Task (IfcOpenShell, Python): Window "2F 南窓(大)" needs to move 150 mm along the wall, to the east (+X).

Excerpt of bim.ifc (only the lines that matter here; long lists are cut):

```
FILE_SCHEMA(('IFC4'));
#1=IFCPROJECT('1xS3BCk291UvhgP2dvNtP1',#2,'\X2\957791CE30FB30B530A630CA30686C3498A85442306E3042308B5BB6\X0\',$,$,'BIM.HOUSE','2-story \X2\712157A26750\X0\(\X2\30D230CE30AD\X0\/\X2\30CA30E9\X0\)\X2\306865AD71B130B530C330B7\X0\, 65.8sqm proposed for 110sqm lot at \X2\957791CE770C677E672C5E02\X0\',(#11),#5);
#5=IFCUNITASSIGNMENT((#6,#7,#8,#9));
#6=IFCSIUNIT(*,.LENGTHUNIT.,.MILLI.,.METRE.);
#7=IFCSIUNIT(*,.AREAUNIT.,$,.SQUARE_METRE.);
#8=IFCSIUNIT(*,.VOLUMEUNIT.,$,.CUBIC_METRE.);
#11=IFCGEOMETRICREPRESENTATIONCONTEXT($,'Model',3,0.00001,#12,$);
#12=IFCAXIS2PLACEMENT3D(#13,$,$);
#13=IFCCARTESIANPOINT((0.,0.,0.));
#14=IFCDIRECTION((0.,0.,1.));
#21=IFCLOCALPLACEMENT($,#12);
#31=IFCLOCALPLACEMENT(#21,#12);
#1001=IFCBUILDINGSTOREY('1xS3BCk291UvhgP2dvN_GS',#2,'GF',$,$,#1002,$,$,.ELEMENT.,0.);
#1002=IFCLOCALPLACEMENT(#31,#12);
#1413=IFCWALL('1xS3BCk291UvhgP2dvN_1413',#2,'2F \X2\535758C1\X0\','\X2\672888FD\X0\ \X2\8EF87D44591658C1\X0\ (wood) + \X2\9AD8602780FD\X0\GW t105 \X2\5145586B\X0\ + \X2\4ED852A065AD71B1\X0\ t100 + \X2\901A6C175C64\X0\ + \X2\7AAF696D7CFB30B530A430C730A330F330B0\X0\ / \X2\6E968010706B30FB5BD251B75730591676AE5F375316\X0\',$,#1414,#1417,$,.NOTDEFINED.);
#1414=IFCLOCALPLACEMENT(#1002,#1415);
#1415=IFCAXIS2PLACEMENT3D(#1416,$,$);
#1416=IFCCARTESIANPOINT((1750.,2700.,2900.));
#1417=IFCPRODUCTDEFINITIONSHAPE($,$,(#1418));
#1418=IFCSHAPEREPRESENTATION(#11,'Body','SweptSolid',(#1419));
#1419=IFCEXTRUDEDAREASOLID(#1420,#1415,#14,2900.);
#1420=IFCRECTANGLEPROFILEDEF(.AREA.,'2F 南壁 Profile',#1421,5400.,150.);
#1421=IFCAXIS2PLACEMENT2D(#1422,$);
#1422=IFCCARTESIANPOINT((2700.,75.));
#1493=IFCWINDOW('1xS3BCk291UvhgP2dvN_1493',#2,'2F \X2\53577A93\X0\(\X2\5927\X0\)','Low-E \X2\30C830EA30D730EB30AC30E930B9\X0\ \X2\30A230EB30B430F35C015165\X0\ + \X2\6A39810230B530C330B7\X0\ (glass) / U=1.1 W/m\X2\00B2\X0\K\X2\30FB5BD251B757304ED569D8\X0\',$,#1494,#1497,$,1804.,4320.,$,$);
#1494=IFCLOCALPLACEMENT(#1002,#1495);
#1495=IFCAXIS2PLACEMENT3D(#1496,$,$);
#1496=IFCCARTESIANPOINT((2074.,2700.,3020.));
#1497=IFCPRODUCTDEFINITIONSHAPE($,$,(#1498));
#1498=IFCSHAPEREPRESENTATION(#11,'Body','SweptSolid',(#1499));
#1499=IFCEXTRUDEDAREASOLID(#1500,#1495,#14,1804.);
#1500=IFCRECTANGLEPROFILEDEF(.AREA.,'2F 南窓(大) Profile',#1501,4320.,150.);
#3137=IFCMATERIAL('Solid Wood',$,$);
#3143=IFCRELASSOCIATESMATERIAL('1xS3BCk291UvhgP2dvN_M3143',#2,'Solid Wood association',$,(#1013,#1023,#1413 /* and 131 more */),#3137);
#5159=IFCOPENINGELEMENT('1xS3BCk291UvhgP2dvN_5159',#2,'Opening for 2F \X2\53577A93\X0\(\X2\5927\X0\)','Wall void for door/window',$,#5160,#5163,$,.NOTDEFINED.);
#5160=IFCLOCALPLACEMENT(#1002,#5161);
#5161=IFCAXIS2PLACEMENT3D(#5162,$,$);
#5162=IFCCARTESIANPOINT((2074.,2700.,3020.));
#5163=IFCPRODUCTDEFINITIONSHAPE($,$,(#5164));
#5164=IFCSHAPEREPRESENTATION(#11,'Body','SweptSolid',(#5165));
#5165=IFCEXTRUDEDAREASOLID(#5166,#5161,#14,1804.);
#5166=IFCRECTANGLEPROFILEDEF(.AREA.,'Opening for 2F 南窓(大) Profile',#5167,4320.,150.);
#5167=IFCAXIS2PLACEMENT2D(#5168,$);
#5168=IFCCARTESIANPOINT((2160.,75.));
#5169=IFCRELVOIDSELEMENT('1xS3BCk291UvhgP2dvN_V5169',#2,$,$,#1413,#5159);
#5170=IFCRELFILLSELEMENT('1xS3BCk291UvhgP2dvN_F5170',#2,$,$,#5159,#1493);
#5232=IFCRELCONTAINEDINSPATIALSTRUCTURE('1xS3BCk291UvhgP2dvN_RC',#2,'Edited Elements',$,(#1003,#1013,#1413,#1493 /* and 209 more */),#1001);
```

```python
import ifcopenshell
import ifcopenshell.api.geometry
import ifcopenshell.util.placement

model = ifcopenshell.open("bim.ifc")

window = model.by_guid("1xS3BCk291UvhgP2dvN_1493")
opening = window.FillsVoids[0].RelatingOpeningElement
wall = opening.VoidsElements[0].RelatingBuildingElement

wall_matrix = ifcopenshell.util.placement.get_local_placement(wall.ObjectPlacement)
shift = wall_matrix[:3, 0] * 150.0
before = ifcopenshell.util.placement.get_local_placement(window.ObjectPlacement)[:3, 3].copy()

# The window is not placed relative to its opening, so move both.
for product in (opening, window):
    matrix = ifcopenshell.util.placement.get_local_placement(product.ObjectPlacement)
    matrix[:3, 3] += shift
    ifcopenshell.api.geometry.edit_object_placement(model, product=product, matrix=matrix, is_si=False)

after = ifcopenshell.util.placement.get_local_placement(window.ObjectPlacement)[:3, 3]
print("window moved by", (after - before).round(3) + 0.0)

model.write("bim_v2.ifc")
```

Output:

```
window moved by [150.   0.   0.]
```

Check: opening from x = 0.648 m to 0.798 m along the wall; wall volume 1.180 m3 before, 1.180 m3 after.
